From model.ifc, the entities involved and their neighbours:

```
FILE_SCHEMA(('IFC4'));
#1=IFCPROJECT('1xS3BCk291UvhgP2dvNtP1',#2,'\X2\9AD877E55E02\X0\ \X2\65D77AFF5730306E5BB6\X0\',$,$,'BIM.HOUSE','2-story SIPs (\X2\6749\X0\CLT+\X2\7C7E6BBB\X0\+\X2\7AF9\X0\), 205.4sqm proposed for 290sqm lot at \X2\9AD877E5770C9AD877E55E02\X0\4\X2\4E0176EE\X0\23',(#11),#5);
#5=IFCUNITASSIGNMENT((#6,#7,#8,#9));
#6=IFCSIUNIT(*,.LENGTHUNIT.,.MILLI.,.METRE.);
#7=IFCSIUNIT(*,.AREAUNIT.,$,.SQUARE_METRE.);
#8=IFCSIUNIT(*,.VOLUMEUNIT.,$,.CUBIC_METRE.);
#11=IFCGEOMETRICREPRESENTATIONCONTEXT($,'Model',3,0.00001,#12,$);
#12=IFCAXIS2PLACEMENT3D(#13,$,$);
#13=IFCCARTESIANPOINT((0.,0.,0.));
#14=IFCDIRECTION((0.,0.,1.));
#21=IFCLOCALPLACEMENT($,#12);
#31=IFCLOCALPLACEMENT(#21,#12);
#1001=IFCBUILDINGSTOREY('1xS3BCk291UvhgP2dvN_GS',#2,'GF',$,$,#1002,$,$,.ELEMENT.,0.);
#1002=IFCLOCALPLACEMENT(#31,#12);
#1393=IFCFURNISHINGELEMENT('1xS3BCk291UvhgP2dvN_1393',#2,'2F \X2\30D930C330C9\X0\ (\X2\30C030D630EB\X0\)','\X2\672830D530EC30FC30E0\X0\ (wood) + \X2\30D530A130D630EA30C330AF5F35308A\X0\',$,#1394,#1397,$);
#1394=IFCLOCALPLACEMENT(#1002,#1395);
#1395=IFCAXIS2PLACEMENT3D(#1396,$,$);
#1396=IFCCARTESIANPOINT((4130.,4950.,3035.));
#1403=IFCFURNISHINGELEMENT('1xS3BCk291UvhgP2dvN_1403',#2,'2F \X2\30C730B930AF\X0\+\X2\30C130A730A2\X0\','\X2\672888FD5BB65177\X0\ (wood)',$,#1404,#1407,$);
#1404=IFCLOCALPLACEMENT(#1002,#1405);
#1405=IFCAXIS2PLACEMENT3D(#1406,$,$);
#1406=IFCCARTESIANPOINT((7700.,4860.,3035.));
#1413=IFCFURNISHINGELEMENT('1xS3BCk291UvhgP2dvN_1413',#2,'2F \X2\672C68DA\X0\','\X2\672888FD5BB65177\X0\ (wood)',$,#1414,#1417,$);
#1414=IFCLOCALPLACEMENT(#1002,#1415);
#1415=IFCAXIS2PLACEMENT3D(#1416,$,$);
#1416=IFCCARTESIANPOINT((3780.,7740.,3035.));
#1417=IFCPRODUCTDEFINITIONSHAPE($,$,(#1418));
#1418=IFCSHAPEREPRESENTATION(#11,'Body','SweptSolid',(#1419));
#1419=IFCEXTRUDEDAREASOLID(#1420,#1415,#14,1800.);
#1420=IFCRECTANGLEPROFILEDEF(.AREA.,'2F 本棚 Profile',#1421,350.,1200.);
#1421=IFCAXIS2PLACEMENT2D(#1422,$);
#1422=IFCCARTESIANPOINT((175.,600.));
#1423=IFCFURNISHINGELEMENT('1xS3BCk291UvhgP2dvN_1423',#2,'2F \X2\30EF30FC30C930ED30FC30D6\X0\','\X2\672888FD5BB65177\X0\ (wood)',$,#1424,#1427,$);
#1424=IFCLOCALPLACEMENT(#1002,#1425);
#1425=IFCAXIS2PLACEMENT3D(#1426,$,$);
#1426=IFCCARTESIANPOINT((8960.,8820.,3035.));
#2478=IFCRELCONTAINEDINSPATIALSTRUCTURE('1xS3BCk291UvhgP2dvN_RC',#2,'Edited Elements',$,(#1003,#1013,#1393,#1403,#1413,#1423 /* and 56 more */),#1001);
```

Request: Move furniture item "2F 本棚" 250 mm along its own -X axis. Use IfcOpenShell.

```python
import ifcopenshell
import ifcopenshell.api.geometry
import ifcopenshell.util.placement
import ifcopenshell.util.unit

model = ifcopenshell.open("model.ifc")
unit_scale = ifcopenshell.util.unit.calculate_unit_scale(model)

item = model.by_guid("1xS3BCk291UvhgP2dvN_1413")
matrix = ifcopenshell.util.placement.get_local_placement(item.ObjectPlacement)
matrix[:3, 3] -= matrix[:3, 0] * 0.25 / unit_scale
ifcopenshell.api.geometry.edit_object_placement(model, product=item, matrix=matrix, is_si=False)

print(ifcopenshell.util.placement.get_local_placement(item.ObjectPlacement).round(3) + 0.0)

model.write("model-out.ifc")
```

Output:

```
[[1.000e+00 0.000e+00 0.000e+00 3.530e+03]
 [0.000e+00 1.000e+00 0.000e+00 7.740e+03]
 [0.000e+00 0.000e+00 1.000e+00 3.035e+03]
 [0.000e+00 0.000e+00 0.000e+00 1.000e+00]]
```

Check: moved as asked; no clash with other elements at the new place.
